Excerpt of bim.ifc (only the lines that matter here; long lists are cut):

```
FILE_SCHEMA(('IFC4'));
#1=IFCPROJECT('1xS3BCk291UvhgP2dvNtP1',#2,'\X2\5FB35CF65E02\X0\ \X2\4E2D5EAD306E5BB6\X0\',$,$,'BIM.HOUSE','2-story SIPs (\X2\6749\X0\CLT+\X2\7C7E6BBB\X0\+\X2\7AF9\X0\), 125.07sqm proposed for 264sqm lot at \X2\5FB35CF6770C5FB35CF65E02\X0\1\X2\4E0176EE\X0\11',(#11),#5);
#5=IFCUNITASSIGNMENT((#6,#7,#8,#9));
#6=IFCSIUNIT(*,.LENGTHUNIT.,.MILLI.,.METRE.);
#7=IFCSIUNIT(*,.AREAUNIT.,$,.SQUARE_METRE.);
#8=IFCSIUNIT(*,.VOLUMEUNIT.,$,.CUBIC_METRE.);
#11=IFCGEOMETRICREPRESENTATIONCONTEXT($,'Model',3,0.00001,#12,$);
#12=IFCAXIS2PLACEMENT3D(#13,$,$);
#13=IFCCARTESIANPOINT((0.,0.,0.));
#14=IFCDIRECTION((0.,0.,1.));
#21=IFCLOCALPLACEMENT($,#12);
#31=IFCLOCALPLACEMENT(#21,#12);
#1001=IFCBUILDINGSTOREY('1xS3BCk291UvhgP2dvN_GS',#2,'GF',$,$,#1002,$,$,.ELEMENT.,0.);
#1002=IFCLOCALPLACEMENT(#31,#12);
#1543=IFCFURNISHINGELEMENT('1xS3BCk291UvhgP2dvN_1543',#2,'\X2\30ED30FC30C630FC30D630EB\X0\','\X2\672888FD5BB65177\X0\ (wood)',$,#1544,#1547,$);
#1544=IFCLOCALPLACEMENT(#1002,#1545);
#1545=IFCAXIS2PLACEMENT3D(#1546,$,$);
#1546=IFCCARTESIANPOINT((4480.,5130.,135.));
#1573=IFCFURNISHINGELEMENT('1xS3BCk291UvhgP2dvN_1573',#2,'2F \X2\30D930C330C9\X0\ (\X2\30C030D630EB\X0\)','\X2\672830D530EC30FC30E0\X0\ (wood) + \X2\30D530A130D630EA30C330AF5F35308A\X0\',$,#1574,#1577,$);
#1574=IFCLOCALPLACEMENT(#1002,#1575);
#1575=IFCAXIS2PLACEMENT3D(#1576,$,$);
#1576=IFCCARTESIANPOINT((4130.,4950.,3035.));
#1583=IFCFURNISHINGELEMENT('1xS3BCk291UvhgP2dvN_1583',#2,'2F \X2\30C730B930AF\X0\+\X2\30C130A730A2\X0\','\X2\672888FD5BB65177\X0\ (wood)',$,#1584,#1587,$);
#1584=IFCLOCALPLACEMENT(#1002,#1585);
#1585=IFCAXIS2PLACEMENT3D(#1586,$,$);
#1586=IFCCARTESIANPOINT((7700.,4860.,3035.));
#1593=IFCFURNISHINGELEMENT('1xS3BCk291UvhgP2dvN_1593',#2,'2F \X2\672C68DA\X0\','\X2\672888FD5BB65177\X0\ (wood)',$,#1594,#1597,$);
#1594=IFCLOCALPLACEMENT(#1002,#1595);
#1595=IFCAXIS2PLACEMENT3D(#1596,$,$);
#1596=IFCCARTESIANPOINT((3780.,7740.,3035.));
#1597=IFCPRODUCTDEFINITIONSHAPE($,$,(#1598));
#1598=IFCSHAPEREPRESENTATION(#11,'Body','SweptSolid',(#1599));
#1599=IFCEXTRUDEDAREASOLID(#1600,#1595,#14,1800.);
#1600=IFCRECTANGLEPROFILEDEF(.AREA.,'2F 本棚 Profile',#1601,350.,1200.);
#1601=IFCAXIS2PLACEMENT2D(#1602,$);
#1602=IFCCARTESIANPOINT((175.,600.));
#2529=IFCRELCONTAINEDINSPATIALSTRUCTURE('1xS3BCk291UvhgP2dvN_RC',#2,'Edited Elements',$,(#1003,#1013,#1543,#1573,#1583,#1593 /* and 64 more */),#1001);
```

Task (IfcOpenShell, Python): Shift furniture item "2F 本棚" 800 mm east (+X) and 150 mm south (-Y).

```python
import ifcopenshell
import ifcopenshell.api.geometry
import ifcopenshell.util.placement
import ifcopenshell.util.unit

model = ifcopenshell.open("bim.ifc")
unit_scale = ifcopenshell.util.unit.calculate_unit_scale(model)

item = model.by_id(1593)
matrix = ifcopenshell.util.placement.get_local_placement(item.ObjectPlacement)
matrix[0, 3] += 0.8 / unit_scale
matrix[1, 3] -= 0.15 / unit_scale
ifcopenshell.api.geometry.edit_object_placement(model, product=item, matrix=matrix, is_si=False)

print(ifcopenshell.util.placement.get_local_placement(item.ObjectPlacement).round(3) + 0.0)

model.write("bim-out.ifc")
```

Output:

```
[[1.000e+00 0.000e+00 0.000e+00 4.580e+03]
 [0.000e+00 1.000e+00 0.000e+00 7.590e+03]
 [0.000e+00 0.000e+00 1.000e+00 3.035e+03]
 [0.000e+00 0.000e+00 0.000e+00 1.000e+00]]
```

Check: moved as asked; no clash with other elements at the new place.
